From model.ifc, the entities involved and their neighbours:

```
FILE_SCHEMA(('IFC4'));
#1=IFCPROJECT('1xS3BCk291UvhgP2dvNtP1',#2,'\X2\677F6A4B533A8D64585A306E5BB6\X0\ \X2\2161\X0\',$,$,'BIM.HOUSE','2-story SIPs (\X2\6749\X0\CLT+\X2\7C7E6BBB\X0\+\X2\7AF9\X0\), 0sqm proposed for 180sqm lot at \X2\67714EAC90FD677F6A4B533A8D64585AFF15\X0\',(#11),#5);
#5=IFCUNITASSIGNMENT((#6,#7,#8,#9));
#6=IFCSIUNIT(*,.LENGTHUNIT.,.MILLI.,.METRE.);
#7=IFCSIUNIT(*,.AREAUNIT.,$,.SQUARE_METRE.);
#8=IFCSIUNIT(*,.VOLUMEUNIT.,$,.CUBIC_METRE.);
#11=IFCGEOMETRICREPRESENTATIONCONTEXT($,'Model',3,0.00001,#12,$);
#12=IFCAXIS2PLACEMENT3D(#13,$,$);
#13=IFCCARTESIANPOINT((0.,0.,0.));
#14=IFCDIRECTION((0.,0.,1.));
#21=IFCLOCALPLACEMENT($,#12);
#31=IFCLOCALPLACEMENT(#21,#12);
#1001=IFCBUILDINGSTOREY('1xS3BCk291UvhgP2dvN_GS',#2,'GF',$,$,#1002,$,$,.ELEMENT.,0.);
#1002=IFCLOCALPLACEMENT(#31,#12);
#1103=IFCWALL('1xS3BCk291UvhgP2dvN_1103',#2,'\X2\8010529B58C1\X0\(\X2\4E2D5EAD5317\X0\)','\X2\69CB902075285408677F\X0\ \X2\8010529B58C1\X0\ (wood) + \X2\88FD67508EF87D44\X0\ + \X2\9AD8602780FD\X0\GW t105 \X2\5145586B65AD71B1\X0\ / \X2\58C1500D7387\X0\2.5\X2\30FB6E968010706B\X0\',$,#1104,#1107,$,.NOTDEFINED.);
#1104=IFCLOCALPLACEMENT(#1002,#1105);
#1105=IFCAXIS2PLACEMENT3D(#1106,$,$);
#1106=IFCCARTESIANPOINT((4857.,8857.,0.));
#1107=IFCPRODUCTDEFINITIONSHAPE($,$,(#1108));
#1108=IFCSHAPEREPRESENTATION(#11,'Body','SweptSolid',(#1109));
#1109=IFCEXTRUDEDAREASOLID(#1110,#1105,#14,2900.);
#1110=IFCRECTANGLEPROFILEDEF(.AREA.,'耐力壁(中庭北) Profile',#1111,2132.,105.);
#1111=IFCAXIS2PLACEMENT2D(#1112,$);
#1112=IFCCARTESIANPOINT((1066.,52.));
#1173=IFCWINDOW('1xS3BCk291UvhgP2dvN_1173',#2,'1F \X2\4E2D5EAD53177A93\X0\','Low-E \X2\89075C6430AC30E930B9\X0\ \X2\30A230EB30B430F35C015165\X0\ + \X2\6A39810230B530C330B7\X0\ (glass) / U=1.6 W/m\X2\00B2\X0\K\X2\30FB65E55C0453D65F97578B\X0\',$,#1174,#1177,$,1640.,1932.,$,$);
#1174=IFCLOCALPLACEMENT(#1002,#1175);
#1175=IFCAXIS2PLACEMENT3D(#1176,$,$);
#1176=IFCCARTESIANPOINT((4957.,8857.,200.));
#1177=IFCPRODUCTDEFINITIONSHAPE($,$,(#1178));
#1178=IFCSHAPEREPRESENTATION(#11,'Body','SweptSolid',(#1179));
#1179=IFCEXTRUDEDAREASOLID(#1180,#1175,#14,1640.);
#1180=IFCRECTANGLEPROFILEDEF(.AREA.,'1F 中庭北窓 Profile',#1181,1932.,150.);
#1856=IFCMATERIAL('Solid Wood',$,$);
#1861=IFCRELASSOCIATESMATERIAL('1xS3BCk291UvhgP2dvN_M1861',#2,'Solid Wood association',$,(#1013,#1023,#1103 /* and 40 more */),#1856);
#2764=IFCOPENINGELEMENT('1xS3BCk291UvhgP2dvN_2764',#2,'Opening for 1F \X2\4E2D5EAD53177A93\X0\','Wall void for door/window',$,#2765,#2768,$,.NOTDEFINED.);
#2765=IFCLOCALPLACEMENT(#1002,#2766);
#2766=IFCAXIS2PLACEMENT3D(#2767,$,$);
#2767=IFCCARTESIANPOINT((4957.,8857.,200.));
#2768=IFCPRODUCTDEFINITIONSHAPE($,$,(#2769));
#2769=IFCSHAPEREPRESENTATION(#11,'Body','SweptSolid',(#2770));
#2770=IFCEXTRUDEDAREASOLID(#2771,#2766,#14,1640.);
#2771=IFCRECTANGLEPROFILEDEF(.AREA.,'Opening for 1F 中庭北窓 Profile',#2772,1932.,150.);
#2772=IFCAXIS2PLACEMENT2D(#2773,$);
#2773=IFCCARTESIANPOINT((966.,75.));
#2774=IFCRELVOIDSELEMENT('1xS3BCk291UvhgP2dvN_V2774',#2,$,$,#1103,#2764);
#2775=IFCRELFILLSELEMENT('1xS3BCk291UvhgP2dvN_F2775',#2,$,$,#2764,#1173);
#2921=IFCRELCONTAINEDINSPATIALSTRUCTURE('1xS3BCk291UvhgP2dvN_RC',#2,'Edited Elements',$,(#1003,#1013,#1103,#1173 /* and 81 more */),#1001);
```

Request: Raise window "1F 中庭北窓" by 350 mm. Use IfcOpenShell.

```python
import numpy as np
import ifcopenshell
import ifcopenshell.api.geometry
import ifcopenshell.util.placement
import ifcopenshell.util.unit

model = ifcopenshell.open("model.ifc")
unit_scale = ifcopenshell.util.unit.calculate_unit_scale(model)

window = model.by_guid("1xS3BCk291UvhgP2dvN_1173")
opening = window.FillsVoids[0].RelatingOpeningElement
dz = 0.35 / unit_scale

shift = np.array([0.0, 0.0, dz])
# The window is not placed relative to its opening, so move both.
for product in (opening, window):
    matrix = ifcopenshell.util.placement.get_local_placement(product.ObjectPlacement)
    matrix[:3, 3] += shift
    ifcopenshell.api.geometry.edit_object_placement(model, product=product, matrix=matrix, is_si=False)

print(f"moved by {dz * unit_scale:+.3f} m")

model.write("model_rev.ifc")
```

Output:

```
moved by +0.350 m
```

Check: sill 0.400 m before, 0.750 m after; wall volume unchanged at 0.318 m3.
